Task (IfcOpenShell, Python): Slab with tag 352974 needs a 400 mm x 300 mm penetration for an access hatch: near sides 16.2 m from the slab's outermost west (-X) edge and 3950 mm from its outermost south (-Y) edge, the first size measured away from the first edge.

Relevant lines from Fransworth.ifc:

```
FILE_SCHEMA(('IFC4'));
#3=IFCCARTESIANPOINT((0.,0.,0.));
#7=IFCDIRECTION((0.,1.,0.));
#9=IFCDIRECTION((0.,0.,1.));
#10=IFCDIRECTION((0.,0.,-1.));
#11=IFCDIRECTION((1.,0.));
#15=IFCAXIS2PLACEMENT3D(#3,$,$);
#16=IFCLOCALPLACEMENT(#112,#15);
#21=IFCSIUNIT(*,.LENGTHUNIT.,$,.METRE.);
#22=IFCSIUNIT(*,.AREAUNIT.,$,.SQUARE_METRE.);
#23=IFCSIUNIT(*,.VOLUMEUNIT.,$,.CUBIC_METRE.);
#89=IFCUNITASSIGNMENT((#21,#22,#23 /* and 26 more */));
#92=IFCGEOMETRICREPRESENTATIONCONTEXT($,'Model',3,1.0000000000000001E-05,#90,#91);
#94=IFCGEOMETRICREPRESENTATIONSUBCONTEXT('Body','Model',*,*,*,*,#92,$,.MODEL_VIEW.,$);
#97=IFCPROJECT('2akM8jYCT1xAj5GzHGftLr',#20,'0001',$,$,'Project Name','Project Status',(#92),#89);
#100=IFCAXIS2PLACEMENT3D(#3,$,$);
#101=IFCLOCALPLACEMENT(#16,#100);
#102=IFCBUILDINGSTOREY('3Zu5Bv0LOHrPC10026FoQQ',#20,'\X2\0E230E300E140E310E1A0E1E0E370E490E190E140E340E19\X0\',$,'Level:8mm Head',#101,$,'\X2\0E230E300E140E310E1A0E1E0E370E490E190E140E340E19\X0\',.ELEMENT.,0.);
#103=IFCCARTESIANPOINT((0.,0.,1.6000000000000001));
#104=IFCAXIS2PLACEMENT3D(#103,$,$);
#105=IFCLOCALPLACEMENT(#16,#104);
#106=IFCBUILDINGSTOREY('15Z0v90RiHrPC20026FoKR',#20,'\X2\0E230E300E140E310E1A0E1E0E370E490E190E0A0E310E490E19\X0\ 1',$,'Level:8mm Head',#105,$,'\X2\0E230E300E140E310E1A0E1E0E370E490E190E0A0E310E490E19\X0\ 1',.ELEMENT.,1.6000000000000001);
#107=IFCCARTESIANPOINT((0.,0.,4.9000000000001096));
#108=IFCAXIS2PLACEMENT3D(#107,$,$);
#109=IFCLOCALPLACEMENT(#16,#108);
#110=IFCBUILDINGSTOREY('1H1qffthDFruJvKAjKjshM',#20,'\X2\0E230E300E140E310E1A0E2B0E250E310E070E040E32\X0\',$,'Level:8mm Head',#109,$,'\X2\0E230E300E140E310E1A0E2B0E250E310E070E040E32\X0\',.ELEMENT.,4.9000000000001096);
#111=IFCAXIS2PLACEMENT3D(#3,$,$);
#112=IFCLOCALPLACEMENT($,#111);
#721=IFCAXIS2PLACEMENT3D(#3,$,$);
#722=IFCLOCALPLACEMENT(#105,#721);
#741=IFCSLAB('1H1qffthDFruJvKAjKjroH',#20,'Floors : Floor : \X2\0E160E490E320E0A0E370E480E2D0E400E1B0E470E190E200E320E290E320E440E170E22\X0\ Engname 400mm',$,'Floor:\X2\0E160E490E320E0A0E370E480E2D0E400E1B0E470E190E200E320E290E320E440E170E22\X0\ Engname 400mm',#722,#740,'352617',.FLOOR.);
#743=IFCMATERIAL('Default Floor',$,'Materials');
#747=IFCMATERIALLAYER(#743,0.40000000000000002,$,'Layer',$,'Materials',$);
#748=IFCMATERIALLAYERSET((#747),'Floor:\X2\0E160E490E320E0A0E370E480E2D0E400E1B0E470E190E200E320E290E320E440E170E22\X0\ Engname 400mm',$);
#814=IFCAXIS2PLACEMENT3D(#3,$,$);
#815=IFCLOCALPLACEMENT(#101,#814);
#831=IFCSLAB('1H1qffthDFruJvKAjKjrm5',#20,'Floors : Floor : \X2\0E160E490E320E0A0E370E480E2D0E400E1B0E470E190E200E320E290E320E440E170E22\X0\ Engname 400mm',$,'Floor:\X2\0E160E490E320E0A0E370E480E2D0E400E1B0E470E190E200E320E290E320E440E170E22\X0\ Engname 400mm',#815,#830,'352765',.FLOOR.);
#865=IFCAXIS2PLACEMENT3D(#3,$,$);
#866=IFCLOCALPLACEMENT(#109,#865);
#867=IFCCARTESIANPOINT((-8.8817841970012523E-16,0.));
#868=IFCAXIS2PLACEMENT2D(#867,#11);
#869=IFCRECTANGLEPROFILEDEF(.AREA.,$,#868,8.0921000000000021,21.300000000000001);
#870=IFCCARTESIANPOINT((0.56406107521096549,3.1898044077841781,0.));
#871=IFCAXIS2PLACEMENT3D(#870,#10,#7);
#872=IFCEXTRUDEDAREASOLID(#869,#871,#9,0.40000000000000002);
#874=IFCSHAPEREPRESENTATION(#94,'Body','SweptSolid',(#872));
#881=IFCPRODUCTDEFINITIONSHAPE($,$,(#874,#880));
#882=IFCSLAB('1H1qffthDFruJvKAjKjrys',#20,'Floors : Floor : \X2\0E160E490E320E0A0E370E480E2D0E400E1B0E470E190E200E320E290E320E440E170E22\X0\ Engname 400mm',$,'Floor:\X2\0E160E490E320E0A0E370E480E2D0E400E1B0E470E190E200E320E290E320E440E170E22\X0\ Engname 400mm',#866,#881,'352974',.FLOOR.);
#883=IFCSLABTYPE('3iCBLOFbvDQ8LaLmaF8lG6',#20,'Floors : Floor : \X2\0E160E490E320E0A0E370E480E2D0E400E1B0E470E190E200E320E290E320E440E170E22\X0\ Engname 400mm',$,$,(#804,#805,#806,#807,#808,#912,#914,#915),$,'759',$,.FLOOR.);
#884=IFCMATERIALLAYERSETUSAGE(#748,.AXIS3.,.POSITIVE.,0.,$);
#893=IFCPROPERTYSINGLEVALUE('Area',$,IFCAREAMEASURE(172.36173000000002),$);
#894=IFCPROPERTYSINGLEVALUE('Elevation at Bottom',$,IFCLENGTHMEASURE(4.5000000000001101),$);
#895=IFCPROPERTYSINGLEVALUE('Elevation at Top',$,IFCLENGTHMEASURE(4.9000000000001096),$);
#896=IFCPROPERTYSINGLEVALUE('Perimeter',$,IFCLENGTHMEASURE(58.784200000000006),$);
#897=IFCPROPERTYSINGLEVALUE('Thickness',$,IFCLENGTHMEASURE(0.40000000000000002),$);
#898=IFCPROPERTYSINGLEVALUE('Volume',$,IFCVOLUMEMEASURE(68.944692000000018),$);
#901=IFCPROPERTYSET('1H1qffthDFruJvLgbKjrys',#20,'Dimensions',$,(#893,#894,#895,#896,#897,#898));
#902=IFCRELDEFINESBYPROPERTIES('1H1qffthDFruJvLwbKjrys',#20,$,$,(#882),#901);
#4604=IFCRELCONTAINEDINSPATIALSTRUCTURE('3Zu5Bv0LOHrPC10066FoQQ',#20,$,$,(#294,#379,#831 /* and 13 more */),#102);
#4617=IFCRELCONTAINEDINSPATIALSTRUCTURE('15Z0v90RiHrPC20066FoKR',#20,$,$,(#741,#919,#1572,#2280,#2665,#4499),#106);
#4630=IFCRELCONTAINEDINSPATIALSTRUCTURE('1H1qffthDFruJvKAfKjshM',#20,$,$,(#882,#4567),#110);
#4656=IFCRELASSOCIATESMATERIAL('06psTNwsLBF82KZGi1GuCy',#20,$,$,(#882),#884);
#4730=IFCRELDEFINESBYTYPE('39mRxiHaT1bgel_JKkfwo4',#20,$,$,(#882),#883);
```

```python
import numpy as np
import ifcopenshell
import ifcopenshell.api.feature
import ifcopenshell.api.geometry
import ifcopenshell.api.pset
import ifcopenshell.api.root
import ifcopenshell.geom
import ifcopenshell.util.element
import ifcopenshell.util.placement
import ifcopenshell.util.representation
import ifcopenshell.util.shape
import ifcopenshell.util.unit

model = ifcopenshell.open("Fransworth.ifc")
unit_scale = ifcopenshell.util.unit.calculate_unit_scale(model)
area_scale = ifcopenshell.util.unit.calculate_unit_scale(model, "AREAUNIT")
volume_scale = ifcopenshell.util.unit.calculate_unit_scale(model, "VOLUMEUNIT")
settings = ifcopenshell.geom.settings()


def volume(element):
    """Net volume in cubic metres, openings subtracted."""
    shape = ifcopenshell.geom.create_shape(settings, element)
    return ifcopenshell.util.shape.get_volume(shape.geometry)


slab = model.by_guid("1H1qffthDFruJvKAjKjrys")
before = volume(slab)

# Extent in the slab's own axes, in metres. The edges named are its -X and -Y sides.
slab_shape = ifcopenshell.geom.create_shape(settings, slab)
vertices = ifcopenshell.util.shape.get_vertices(slab_shape.geometry)
x_min, y_min, bottom = vertices.min(axis=0)
top = vertices[:, 2].max()

opening = ifcopenshell.api.root.create_entity(model, ifc_class="IfcOpeningElement", name="Access hatch opening", predefined_type="OPENING")
context = ifcopenshell.util.representation.get_context(model, "Model", "Body", "MODEL_VIEW")
width, depth = 0.4, 0.3
outline = [(0.0, 0.0), (width, 0.0), (width, depth), (0.0, depth), (0.0, 0.0)]
# Overshoot both faces by 50 mm so the cut is clean.
shape = ifcopenshell.api.geometry.add_slab_representation(
    model, context=context, depth=top - bottom + 0.1, polyline=outline
)
ifcopenshell.api.geometry.assign_representation(model, product=opening, representation=shape)

matrix = ifcopenshell.util.placement.get_local_placement(slab.ObjectPlacement)
matrix[:, 3] = matrix @ np.append(np.array([x_min + 16.2, y_min + 3.95, bottom - 0.05]) / unit_scale, 1.0)
ifcopenshell.api.geometry.edit_object_placement(model, product=opening, matrix=matrix, is_si=False)
ifcopenshell.api.feature.add_feature(model, feature=opening, element=slab)

after = volume(slab)

# Update the slab's stored quantities.
pset = model.by_id(ifcopenshell.util.element.get_pset(slab, "Dimensions", should_inherit=False)["id"])
ifcopenshell.api.pset.edit_pset(model, pset=pset, properties={
    "Area": model.create_entity("IfcAreaMeasure", after / (top - bottom) / area_scale),
    "Volume": model.create_entity("IfcVolumeMeasure", after / volume_scale),
})

print(f"slab volume {before:.3f} -> {after:.3f} m3")

model.write("Fransworth_v2.ifc")
```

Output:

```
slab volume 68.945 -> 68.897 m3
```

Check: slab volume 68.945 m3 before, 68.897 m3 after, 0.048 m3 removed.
